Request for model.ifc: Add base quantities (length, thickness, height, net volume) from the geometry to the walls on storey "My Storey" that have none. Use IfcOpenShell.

First a look at what the model holds.

```python
import ifcopenshell
import ifcopenshell.util.element
import ifcopenshell.util.unit

model = ifcopenshell.open("model.ifc")
print(model.schema)
for unit_type in ("LENGTHUNIT", "AREAUNIT", "VOLUMEUNIT"):
    print(unit_type, ifcopenshell.util.unit.calculate_unit_scale(model, unit_type))
storey = next(s for s in model.by_type("IfcBuildingStorey") if s.Name == "My Storey")
walls = [e for e in ifcopenshell.util.element.get_decomposition(storey) if e.is_a("IfcWall")]
for e in sorted(walls, key=lambda e: e.id()):
    print(e.id(), e.is_a(), e.Name, list(ifcopenshell.util.element.get_psets(e, qtos_only=True)), sep=" | ")
```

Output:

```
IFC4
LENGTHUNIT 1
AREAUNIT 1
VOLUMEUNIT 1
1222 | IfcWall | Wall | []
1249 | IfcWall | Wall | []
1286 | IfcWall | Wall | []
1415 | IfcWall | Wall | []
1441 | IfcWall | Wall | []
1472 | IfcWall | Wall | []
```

```python
import ifcopenshell
import ifcopenshell.api.pset
import ifcopenshell.geom
import ifcopenshell.util.element
import ifcopenshell.util.shape
import ifcopenshell.util.unit

model = ifcopenshell.open("model.ifc")
unit_scale = ifcopenshell.util.unit.calculate_unit_scale(model)
volume_scale = ifcopenshell.util.unit.calculate_unit_scale(model, "VOLUMEUNIT")
settings = ifcopenshell.geom.settings()

storey = next(s for s in model.by_type("IfcBuildingStorey") if s.Name == "My Storey")
walls = [e for e in ifcopenshell.util.element.get_decomposition(storey) if e.is_a("IfcWall")]

for e in sorted(walls, key=lambda e: e.id()):
    if ifcopenshell.util.element.get_psets(e, qtos_only=True, should_inherit=False):
        continue
    # Geometry comes back in metres, in the element's own axes.
    shape = ifcopenshell.geom.create_shape(settings, e)
    values = {
        "Length": ifcopenshell.util.shape.get_x(shape.geometry) / unit_scale,
        "Width": ifcopenshell.util.shape.get_y(shape.geometry) / unit_scale,
        "Height": ifcopenshell.util.shape.get_z(shape.geometry) / unit_scale,
        "NetVolume": ifcopenshell.util.shape.get_volume(shape.geometry) / volume_scale,
    }
    qto = ifcopenshell.api.pset.add_qto(model, product=e, name="Qto_WallBaseQuantities")
    ifcopenshell.api.pset.edit_qto(model, qto=qto, properties=values)
    print(e.id(), {k: round(v, 3) for k, v in values.items()})

model.write("model_updated.ifc")
```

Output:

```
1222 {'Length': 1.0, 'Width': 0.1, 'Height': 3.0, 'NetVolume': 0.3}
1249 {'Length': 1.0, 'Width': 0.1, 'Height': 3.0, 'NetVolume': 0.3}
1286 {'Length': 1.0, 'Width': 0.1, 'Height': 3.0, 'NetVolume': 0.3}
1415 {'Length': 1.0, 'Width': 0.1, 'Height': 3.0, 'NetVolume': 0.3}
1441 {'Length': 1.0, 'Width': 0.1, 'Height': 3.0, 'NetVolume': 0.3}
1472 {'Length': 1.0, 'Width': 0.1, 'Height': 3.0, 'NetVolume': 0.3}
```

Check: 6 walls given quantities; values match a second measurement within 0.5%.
